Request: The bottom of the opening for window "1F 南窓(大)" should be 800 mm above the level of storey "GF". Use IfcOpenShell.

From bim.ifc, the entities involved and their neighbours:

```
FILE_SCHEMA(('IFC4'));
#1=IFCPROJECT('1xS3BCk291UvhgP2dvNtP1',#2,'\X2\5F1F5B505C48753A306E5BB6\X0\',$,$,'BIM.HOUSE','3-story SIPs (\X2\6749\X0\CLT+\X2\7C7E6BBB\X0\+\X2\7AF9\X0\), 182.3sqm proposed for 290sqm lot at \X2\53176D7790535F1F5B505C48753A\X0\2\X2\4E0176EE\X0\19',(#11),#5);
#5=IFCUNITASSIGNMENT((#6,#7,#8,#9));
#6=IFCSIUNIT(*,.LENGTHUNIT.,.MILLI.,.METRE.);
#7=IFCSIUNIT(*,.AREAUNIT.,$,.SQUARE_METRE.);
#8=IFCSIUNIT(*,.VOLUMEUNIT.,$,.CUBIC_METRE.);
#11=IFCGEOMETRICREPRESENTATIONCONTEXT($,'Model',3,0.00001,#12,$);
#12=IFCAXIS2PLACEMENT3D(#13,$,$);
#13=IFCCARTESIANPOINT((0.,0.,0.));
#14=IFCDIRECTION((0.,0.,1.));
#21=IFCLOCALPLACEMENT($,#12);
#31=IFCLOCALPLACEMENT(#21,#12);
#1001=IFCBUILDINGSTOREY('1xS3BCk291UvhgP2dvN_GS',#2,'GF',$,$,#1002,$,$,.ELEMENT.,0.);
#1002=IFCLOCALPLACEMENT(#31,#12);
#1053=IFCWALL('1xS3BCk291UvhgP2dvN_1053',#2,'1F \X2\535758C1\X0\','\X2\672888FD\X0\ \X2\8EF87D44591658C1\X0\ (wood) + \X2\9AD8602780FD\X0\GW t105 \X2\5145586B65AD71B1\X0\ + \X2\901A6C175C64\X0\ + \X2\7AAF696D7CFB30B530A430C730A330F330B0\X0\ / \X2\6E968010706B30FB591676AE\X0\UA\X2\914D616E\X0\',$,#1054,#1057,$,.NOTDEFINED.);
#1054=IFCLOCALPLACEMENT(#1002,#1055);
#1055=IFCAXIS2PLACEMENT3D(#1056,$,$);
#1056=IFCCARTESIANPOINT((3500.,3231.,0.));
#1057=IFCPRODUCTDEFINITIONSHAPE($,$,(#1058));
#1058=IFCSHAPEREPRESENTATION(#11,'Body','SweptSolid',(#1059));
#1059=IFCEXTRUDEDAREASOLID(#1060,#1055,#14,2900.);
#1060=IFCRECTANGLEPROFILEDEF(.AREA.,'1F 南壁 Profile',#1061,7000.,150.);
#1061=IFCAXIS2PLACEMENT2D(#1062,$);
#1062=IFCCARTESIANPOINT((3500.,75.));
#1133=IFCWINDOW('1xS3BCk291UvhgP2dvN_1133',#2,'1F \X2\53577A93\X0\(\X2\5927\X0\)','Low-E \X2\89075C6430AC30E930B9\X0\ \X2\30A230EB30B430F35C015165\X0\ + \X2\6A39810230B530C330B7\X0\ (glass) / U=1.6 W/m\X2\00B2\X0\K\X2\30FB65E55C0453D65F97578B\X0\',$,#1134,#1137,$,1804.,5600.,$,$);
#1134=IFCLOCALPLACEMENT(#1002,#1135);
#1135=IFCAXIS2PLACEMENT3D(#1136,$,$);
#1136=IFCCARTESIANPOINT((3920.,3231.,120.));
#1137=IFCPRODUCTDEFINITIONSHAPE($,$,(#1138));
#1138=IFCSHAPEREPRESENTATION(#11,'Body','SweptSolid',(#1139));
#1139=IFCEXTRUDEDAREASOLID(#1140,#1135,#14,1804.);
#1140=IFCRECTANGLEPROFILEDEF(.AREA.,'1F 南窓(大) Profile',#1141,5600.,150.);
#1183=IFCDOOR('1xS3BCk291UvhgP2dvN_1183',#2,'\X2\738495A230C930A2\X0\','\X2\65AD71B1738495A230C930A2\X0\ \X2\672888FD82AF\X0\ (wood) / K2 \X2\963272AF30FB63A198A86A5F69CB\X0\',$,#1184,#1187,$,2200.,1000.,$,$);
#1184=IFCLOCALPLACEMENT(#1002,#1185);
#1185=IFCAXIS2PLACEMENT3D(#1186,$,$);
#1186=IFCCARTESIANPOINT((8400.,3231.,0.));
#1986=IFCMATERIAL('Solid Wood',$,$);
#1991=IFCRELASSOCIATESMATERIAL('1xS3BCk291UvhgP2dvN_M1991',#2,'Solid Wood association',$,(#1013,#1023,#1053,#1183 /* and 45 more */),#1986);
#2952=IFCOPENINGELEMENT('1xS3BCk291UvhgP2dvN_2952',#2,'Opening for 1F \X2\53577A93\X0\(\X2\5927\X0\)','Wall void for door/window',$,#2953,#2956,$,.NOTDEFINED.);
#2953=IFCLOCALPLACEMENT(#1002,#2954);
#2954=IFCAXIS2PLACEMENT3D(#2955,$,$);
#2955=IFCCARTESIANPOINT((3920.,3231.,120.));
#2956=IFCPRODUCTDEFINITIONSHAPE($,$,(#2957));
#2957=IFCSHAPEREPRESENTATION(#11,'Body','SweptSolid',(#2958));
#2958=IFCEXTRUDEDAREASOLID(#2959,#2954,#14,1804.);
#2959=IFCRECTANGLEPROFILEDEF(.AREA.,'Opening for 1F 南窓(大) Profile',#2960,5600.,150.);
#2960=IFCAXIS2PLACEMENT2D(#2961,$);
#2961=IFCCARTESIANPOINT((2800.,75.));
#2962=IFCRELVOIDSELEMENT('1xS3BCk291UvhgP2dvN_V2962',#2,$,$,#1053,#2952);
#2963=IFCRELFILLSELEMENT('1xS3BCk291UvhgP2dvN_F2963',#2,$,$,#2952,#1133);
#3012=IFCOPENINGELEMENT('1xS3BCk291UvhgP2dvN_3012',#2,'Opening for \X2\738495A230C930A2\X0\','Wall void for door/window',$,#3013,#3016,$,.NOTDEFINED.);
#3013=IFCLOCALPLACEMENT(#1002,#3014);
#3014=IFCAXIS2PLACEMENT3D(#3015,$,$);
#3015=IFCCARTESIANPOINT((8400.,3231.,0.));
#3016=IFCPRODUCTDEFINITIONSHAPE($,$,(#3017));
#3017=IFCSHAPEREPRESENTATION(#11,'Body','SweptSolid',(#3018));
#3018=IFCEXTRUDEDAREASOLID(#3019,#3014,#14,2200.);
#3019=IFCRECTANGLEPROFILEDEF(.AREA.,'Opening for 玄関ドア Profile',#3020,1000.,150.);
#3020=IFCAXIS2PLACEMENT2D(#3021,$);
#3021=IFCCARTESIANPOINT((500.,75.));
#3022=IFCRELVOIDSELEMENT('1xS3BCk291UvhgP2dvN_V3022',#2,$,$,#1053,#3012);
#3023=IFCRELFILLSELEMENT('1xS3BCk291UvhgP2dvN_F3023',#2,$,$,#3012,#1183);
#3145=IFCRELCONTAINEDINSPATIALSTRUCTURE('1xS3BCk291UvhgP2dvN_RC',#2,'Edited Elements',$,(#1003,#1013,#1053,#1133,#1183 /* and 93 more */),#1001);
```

```python
import numpy as np
import ifcopenshell
import ifcopenshell.api.geometry
import ifcopenshell.geom
import ifcopenshell.util.element
import ifcopenshell.util.placement
import ifcopenshell.util.shape
import ifcopenshell.util.unit

model = ifcopenshell.open("bim.ifc")
unit_scale = ifcopenshell.util.unit.calculate_unit_scale(model)

window = model.by_guid("1xS3BCk291UvhgP2dvN_1133")
opening = window.FillsVoids[0].RelatingOpeningElement
storey = ifcopenshell.util.element.get_container(window, ifc_class="IfcBuildingStorey")
level = ifcopenshell.util.placement.get_local_placement(storey.ObjectPlacement)[2, 3]

# The opening's origin need not be at the sill, so measure its lowest point.
shape = ifcopenshell.geom.create_shape(ifcopenshell.geom.settings(), opening)
bottom = ifcopenshell.util.shape.get_shape_bottom_elevation(shape, shape.geometry) / unit_scale
dz = level + 0.8 / unit_scale - bottom

shift = np.array([0.0, 0.0, dz])
# The window is not placed relative to its opening, so move both.
for product in (opening, window):
    matrix = ifcopenshell.util.placement.get_local_placement(product.ObjectPlacement)
    matrix[:3, 3] += shift
    ifcopenshell.api.geometry.edit_object_placement(model, product=product, matrix=matrix, is_si=False)

print(f"moved by {dz * unit_scale:+.3f} m")

model.write("bim_updated.ifc")
```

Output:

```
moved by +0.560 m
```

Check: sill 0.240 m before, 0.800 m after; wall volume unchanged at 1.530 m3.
